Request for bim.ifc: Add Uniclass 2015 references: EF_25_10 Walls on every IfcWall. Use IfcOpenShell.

First a look at what the model holds.

```python
import ifcopenshell

model = ifcopenshell.open("bim.ifc")
print(model.schema)
print("classifications:", [c.Name for c in model.by_type("IfcClassification")])
for ifc_class in ("IfcDoor", "IfcRoof", "IfcStair", "IfcWall", "IfcWindow"):
    print(ifc_class, len(model.by_type(ifc_class)))
```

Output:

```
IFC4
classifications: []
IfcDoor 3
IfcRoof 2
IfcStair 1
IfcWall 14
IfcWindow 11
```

```python
import ifcopenshell
import ifcopenshell.api.classification

model = ifcopenshell.open("bim.ifc")

system = ifcopenshell.api.classification.add_classification(model, classification="Uniclass 2015")

codes = {
    "IfcWall": ("EF_25_10", "Walls"),
}
for ifc_class, (code, name) in codes.items():
    products = model.by_type(ifc_class)
    ifcopenshell.api.classification.add_reference(
        model, products=products, classification=system, identification=code, name=name
    )
    print(code, len(products))

model.write("bim-out.ifc")
```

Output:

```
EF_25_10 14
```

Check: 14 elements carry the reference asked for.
